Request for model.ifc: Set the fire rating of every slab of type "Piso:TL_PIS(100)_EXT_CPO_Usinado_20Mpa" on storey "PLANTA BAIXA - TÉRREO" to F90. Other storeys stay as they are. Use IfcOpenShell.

First a look at what the model holds.

```python
import ifcopenshell
import ifcopenshell.util.element

model = ifcopenshell.open("model.ifc")
print(model.schema)
storey = next(s for s in model.by_type("IfcBuildingStorey") if s.Name == "PLANTA BAIXA - TÉRREO")
slabs = [e for e in ifcopenshell.util.element.get_decomposition(storey) if e.is_a("IfcSlab")]
seen = {}
for e in slabs:
    element_type = ifcopenshell.util.element.get_type(e)
    key = (element_type.Name if element_type != e and element_type else None, ifcopenshell.util.element.get_pset(e, "Pset_SlabCommon", "FireRating"))
    seen[key] = seen.get(key, 0) + 1
for (name, value), count in sorted(seen.items(), key=str):
    print(count, "x", name, "|", value)
```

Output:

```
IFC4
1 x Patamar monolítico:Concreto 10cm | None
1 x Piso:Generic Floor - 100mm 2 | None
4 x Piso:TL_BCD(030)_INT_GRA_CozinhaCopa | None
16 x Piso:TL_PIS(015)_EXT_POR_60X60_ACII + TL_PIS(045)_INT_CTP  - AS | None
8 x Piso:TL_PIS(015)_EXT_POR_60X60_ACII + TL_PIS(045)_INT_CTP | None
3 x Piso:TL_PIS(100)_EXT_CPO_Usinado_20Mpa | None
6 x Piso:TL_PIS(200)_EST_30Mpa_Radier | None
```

```python
import ifcopenshell
import ifcopenshell.api.pset
import ifcopenshell.util.element

model = ifcopenshell.open("model.ifc")

storey = next(s for s in model.by_type("IfcBuildingStorey") if s.Name == "PLANTA BAIXA - TÉRREO")
slabs = [e for e in ifcopenshell.util.element.get_decomposition(storey) if e.is_a("IfcSlab")]

count = 0
for e in slabs:
    element_type = ifcopenshell.util.element.get_type(e)
    if element_type in (None, e) or element_type.Name != "Piso:TL_PIS(100)_EXT_CPO_Usinado_20Mpa":
        continue
    # add_pset returns the element's existing set when there is one.
    pset = ifcopenshell.api.pset.add_pset(model, product=e, name="Pset_SlabCommon")
    ifcopenshell.api.pset.edit_pset(model, pset=pset, properties={"FireRating": "F90"})
    count += 1

print(count, "slabs updated")

model.write("model_rev.ifc")
```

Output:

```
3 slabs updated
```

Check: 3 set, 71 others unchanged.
